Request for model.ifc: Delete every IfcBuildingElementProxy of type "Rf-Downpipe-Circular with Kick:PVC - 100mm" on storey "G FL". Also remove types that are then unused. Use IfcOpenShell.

First a look at what the model holds.

```python
import ifcopenshell
import ifcopenshell.util.element

model = ifcopenshell.open("model.ifc")
print(model.schema)
storey = next(s for s in model.by_type("IfcBuildingStorey") if s.Name == "G FL")
proxies = [e for e in ifcopenshell.util.element.get_decomposition(storey) if e.is_a("IfcBuildingElementProxy")]
seen = {}
for e in proxies:
    element_type = ifcopenshell.util.element.get_type(e)
    name = element_type.Name if element_type not in (None, e) else None
    seen[name] = seen.get(name, 0) + 1
for name, count in sorted(seen.items(), key=str):
    print(count, "x", name)
```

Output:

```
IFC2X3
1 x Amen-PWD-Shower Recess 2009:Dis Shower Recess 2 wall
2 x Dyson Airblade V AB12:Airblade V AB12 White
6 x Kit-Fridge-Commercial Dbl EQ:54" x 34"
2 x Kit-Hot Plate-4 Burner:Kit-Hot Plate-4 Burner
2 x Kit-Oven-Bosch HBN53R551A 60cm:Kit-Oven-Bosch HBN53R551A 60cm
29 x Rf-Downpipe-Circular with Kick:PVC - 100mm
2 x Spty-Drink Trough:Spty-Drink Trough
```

```python
import ifcopenshell
import ifcopenshell.api.root
import ifcopenshell.util.element

model = ifcopenshell.open("model.ifc")

storey = next(s for s in model.by_type("IfcBuildingStorey") if s.Name == "G FL")
proxies = [e for e in ifcopenshell.util.element.get_decomposition(storey) if e.is_a("IfcBuildingElementProxy")]
targets = [e for e in proxies if (t := ifcopenshell.util.element.get_type(e)) not in (None, e) and t.Name == "Rf-Downpipe-Circular with Kick:PVC - 100mm"]
types = {ifcopenshell.util.element.get_type(e) for e in targets} - {None, *targets}

for e in targets:
    ifcopenshell.api.root.remove_product(model, product=e)
print(len(targets), "removed")

unused = [t for t in types if not ifcopenshell.util.element.get_types(t)]
for t in unused:
    ifcopenshell.api.root.remove_product(model, product=t)
print(len(unused), "unused types removed")

model.write("model_rev.ifc")
```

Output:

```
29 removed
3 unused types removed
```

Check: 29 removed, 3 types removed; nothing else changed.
